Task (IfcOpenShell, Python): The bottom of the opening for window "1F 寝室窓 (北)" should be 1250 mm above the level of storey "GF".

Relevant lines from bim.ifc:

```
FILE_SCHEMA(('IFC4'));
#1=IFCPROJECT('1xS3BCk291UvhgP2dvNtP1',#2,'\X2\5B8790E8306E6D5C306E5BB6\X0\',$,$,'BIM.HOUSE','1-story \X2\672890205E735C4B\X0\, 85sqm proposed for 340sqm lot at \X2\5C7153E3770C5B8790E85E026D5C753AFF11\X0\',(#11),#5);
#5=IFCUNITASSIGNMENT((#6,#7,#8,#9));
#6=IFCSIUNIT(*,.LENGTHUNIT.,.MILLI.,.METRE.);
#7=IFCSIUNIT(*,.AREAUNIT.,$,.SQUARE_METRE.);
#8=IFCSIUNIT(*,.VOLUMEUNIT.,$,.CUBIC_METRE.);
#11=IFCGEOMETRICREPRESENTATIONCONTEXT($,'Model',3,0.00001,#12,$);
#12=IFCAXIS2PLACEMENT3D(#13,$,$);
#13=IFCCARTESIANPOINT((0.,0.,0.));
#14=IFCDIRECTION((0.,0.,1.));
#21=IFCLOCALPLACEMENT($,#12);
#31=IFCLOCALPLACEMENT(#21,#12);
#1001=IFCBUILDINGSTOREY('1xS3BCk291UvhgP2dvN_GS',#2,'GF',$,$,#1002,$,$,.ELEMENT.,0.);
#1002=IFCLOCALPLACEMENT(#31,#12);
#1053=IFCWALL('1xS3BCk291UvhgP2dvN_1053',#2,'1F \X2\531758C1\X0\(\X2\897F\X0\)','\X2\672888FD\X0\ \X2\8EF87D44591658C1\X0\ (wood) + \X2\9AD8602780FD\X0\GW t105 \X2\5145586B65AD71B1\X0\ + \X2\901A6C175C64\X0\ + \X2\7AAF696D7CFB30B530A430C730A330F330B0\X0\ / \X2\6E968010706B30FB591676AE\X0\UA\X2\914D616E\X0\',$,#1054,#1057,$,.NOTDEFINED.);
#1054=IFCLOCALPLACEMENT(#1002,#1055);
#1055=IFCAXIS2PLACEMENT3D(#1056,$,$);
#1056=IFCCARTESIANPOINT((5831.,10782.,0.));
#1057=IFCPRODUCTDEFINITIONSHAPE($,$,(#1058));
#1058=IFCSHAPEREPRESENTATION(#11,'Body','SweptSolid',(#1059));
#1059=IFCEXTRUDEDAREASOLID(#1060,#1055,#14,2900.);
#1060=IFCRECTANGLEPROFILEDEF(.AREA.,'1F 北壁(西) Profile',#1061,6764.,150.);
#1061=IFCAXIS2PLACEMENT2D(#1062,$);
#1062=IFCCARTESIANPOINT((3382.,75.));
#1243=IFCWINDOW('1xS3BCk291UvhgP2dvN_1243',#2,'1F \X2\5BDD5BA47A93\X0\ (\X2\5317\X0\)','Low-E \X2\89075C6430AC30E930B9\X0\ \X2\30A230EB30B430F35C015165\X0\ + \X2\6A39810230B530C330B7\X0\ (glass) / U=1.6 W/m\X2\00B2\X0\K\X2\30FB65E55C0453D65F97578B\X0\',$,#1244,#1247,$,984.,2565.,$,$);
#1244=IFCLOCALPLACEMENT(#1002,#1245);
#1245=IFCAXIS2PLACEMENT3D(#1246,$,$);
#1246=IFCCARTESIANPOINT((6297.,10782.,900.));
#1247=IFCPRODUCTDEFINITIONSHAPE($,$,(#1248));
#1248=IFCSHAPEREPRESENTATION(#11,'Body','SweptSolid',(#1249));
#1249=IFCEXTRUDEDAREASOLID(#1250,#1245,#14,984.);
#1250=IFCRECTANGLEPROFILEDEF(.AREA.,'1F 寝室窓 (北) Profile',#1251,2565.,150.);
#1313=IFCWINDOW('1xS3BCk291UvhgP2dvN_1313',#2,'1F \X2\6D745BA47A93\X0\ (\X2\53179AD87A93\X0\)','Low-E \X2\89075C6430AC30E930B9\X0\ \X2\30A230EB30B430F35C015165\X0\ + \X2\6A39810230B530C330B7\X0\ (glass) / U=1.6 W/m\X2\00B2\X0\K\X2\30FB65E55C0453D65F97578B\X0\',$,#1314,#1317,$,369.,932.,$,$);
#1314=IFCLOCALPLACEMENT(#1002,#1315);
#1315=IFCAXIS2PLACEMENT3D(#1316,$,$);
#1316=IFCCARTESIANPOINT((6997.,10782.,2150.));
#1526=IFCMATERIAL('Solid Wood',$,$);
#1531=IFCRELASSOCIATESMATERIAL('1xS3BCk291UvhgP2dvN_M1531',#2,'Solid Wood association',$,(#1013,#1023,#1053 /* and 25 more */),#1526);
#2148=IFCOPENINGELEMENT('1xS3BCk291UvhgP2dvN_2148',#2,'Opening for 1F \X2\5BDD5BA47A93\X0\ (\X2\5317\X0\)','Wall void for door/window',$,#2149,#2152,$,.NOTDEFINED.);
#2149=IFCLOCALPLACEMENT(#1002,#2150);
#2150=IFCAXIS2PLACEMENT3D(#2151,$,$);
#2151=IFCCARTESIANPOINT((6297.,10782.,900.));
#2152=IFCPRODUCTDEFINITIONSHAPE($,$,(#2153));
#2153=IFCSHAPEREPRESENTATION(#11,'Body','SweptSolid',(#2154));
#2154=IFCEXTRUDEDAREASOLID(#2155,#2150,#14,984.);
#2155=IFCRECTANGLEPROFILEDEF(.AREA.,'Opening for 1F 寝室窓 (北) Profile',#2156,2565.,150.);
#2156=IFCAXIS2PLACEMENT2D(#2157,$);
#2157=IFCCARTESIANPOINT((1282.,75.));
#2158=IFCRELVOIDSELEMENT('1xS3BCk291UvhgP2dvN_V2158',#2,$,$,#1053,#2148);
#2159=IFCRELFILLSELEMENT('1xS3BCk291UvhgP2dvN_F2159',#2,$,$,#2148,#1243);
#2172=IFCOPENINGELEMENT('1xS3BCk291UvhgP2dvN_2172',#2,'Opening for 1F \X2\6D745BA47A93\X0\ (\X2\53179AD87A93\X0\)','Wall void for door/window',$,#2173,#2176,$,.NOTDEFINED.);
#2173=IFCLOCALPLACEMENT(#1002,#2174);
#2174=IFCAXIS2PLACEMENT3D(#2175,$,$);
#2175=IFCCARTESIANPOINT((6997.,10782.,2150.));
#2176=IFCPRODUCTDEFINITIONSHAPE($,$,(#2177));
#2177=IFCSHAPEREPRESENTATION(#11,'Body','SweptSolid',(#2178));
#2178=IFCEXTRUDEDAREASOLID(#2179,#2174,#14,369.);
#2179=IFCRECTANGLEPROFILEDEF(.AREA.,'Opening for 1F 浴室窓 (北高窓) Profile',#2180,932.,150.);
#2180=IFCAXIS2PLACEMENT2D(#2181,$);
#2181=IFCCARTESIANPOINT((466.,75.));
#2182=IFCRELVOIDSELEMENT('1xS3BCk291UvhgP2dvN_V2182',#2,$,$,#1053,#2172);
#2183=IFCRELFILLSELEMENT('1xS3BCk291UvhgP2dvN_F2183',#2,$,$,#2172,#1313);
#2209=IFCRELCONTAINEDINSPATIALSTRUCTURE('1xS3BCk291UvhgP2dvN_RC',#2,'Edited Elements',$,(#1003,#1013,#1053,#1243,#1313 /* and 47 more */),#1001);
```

```python
import numpy as np
import ifcopenshell
import ifcopenshell.api.geometry
import ifcopenshell.geom
import ifcopenshell.util.element
import ifcopenshell.util.placement
import ifcopenshell.util.shape
import ifcopenshell.util.unit

model = ifcopenshell.open("bim.ifc")
unit_scale = ifcopenshell.util.unit.calculate_unit_scale(model)

window = model.by_id(1243)
opening = window.FillsVoids[0].RelatingOpeningElement
storey = ifcopenshell.util.element.get_container(window, ifc_class="IfcBuildingStorey")
level = ifcopenshell.util.placement.get_local_placement(storey.ObjectPlacement)[2, 3]

# The opening's origin need not be at the sill, so measure its lowest point.
shape = ifcopenshell.geom.create_shape(ifcopenshell.geom.settings(), opening)
bottom = ifcopenshell.util.shape.get_shape_bottom_elevation(shape, shape.geometry) / unit_scale
dz = level + 1.25 / unit_scale - bottom

shift = np.array([0.0, 0.0, dz])
# The window is not placed relative to its opening, so move both.
for product in (opening, window):
    matrix = ifcopenshell.util.placement.get_local_placement(product.ObjectPlacement)
    matrix[:3, 3] += shift
    ifcopenshell.api.geometry.edit_object_placement(model, product=product, matrix=matrix, is_si=False)

print(f"moved by {dz * unit_scale:+.3f} m")

model.write("bim_v2.ifc")
```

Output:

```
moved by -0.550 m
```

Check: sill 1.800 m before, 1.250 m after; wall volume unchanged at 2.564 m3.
